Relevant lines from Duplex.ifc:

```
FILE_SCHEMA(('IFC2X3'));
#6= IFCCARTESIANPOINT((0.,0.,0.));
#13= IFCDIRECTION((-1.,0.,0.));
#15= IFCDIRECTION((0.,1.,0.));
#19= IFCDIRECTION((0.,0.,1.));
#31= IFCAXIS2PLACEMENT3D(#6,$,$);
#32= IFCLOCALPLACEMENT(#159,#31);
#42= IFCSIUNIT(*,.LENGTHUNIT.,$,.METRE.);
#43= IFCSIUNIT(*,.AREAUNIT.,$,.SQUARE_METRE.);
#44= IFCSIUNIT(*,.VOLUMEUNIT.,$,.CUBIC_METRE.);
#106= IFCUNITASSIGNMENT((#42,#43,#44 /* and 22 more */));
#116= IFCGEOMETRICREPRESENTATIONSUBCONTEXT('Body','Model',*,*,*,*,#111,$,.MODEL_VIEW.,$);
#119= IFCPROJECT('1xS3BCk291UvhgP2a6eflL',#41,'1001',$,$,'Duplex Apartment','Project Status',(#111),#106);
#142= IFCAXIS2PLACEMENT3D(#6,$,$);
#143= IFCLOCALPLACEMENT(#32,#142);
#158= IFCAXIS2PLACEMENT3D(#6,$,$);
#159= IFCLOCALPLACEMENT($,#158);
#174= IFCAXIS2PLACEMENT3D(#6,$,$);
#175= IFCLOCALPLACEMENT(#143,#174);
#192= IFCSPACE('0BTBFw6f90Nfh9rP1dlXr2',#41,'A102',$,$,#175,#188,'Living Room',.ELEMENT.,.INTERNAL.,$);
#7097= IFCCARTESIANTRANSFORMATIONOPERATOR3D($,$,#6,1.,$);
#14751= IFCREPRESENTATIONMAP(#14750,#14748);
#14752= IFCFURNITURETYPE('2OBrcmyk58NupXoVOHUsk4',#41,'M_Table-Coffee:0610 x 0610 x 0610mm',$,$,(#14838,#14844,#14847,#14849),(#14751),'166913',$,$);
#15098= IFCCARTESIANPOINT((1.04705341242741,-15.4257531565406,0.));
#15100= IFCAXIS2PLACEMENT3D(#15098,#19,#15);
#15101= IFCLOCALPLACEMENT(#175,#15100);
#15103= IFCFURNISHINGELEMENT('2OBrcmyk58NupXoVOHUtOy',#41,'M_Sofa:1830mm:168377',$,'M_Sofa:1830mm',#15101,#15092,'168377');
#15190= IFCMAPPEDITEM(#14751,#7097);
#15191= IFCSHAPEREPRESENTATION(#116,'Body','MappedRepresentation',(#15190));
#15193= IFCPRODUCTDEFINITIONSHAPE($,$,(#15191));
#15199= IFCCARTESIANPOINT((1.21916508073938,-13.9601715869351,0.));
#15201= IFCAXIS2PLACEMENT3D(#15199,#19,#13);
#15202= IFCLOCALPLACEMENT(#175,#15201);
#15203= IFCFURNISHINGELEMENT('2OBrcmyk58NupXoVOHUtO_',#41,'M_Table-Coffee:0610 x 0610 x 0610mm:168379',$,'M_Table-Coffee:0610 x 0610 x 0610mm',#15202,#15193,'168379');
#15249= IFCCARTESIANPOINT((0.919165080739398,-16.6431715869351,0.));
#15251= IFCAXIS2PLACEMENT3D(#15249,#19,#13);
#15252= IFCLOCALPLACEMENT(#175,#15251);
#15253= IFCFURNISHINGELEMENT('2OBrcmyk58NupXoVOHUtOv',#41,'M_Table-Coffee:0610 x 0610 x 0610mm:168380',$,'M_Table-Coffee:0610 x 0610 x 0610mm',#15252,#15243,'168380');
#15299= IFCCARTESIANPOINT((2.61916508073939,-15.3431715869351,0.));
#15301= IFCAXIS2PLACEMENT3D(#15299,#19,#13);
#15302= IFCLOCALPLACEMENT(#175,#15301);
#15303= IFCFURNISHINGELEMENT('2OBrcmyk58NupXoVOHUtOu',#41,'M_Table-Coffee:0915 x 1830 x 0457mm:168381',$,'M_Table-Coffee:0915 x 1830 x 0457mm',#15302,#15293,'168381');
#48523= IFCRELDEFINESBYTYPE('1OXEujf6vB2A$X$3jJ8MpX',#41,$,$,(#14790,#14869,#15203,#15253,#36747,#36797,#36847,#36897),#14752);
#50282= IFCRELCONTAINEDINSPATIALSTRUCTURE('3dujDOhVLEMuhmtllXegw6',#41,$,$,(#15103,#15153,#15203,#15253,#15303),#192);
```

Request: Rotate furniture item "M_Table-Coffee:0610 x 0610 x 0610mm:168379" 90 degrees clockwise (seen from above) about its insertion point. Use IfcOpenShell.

```python
import ifcopenshell
import ifcopenshell.api.geometry
import ifcopenshell.util.placement

model = ifcopenshell.open("Duplex.ifc")

item = model.by_id(15203)
matrix = ifcopenshell.util.placement.get_local_placement(item.ObjectPlacement)
matrix = matrix @ ifcopenshell.util.placement.rotation(-90, "Z")
ifcopenshell.api.geometry.edit_object_placement(model, product=item, matrix=matrix, is_si=False)

print(ifcopenshell.util.placement.get_local_placement(item.ObjectPlacement).round(3) + 0.0)

model.write("Duplex_updated.ifc")
```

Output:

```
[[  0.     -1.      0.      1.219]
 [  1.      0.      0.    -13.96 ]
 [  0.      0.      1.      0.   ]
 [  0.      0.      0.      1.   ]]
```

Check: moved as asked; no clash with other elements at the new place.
